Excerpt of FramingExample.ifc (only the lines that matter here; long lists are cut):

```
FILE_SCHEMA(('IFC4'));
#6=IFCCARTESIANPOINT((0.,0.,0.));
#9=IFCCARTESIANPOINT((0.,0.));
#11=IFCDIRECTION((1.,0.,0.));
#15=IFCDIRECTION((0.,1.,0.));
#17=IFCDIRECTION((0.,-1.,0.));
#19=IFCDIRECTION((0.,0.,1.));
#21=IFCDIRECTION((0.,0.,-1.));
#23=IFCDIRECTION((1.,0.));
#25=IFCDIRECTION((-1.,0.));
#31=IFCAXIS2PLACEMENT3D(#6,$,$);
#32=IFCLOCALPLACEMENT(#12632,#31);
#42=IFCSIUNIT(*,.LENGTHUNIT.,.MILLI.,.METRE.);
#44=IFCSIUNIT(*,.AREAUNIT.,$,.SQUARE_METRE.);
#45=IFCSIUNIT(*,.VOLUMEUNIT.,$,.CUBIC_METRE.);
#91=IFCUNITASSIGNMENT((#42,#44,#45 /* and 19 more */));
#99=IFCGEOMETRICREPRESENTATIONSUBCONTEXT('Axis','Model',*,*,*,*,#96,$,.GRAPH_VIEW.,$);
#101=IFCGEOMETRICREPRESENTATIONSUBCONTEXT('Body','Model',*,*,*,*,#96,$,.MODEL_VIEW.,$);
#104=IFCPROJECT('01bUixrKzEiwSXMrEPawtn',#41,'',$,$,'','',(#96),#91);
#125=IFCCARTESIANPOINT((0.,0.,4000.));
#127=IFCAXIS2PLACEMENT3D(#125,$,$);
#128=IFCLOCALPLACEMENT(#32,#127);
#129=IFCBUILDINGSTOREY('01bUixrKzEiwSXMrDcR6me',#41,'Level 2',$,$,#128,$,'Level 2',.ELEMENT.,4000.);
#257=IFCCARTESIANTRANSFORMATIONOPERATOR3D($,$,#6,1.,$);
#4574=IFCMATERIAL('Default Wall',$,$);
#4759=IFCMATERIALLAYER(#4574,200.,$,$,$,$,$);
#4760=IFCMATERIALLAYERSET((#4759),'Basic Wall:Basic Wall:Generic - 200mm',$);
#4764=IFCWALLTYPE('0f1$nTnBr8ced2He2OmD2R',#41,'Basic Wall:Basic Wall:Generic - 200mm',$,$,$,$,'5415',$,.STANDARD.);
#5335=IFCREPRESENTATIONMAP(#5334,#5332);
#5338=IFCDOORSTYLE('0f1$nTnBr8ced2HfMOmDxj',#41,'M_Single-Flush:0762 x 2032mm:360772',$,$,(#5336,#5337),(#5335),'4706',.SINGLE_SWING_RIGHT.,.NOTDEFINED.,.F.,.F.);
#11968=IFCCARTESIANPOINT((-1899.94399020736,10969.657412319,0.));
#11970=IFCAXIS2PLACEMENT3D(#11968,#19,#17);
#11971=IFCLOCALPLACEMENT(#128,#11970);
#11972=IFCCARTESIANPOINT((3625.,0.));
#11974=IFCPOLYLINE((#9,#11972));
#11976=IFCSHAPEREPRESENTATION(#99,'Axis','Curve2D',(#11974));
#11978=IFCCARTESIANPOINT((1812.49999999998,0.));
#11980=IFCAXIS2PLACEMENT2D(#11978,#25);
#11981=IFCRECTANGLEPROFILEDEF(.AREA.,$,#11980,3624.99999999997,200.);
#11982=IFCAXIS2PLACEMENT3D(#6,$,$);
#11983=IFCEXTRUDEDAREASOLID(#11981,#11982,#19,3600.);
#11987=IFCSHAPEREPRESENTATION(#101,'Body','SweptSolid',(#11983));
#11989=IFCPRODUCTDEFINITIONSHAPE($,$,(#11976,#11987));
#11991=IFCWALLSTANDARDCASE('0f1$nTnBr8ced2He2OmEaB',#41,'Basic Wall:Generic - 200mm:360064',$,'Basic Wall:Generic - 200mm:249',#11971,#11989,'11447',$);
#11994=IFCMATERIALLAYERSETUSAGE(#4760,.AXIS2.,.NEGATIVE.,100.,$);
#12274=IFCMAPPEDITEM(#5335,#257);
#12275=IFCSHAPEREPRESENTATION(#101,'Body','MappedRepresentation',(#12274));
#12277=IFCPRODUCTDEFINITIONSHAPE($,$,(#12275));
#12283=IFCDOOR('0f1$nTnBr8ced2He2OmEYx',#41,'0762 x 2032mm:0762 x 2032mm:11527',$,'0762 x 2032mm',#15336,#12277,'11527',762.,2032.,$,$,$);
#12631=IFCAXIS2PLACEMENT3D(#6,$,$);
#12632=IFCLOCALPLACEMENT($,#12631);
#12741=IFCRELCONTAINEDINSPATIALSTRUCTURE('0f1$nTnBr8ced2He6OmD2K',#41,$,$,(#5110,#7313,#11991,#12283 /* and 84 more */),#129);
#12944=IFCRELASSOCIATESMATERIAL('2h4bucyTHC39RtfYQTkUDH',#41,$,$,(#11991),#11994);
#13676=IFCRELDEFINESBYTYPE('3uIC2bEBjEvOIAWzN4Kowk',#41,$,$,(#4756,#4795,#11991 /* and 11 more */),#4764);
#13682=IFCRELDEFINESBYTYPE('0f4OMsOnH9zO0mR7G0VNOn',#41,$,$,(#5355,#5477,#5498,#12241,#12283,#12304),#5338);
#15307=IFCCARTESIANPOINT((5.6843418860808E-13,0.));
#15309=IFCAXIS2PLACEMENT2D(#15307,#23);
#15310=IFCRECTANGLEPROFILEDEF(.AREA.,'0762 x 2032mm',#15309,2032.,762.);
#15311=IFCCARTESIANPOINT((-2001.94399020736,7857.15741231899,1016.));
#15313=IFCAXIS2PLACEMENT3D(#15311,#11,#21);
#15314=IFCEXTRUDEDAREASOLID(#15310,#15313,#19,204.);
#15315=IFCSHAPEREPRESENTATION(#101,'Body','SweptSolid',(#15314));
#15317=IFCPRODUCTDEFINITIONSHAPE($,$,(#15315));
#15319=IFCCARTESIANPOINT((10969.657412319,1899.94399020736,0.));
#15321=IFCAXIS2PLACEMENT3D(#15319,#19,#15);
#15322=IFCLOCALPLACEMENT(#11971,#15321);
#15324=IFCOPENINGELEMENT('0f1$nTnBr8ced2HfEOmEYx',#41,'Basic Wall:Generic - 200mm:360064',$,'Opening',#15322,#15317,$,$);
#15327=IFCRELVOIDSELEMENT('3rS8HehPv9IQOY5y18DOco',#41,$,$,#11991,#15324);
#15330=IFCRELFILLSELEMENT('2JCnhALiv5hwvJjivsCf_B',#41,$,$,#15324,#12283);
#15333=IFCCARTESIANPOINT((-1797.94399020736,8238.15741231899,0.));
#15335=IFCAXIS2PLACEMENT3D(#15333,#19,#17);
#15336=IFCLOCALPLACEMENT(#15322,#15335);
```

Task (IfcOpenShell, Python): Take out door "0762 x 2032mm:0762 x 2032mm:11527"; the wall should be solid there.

```python
import ifcopenshell
import ifcopenshell.api.feature
import ifcopenshell.api.root
import ifcopenshell.geom
import ifcopenshell.util.shape

model = ifcopenshell.open("FramingExample.ifc")
settings = ifcopenshell.geom.settings()


def volume(element):
    """Net volume in cubic metres, openings subtracted."""
    shape = ifcopenshell.geom.create_shape(settings, element)
    return ifcopenshell.util.shape.get_volume(shape.geometry)


door = model.by_id(12283)
opening = door.FillsVoids[0].RelatingOpeningElement
wall = opening.VoidsElements[0].RelatingBuildingElement
before = volume(wall)

ifcopenshell.api.root.remove_product(model, product=door)
ifcopenshell.api.feature.remove_feature(model, feature=opening)

after = volume(wall)

print(f"wall volume {before:.3f} -> {after:.3f} m3")

model.write("FramingExample_v2.ifc")
```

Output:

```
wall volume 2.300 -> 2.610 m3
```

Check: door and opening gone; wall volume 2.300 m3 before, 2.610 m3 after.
